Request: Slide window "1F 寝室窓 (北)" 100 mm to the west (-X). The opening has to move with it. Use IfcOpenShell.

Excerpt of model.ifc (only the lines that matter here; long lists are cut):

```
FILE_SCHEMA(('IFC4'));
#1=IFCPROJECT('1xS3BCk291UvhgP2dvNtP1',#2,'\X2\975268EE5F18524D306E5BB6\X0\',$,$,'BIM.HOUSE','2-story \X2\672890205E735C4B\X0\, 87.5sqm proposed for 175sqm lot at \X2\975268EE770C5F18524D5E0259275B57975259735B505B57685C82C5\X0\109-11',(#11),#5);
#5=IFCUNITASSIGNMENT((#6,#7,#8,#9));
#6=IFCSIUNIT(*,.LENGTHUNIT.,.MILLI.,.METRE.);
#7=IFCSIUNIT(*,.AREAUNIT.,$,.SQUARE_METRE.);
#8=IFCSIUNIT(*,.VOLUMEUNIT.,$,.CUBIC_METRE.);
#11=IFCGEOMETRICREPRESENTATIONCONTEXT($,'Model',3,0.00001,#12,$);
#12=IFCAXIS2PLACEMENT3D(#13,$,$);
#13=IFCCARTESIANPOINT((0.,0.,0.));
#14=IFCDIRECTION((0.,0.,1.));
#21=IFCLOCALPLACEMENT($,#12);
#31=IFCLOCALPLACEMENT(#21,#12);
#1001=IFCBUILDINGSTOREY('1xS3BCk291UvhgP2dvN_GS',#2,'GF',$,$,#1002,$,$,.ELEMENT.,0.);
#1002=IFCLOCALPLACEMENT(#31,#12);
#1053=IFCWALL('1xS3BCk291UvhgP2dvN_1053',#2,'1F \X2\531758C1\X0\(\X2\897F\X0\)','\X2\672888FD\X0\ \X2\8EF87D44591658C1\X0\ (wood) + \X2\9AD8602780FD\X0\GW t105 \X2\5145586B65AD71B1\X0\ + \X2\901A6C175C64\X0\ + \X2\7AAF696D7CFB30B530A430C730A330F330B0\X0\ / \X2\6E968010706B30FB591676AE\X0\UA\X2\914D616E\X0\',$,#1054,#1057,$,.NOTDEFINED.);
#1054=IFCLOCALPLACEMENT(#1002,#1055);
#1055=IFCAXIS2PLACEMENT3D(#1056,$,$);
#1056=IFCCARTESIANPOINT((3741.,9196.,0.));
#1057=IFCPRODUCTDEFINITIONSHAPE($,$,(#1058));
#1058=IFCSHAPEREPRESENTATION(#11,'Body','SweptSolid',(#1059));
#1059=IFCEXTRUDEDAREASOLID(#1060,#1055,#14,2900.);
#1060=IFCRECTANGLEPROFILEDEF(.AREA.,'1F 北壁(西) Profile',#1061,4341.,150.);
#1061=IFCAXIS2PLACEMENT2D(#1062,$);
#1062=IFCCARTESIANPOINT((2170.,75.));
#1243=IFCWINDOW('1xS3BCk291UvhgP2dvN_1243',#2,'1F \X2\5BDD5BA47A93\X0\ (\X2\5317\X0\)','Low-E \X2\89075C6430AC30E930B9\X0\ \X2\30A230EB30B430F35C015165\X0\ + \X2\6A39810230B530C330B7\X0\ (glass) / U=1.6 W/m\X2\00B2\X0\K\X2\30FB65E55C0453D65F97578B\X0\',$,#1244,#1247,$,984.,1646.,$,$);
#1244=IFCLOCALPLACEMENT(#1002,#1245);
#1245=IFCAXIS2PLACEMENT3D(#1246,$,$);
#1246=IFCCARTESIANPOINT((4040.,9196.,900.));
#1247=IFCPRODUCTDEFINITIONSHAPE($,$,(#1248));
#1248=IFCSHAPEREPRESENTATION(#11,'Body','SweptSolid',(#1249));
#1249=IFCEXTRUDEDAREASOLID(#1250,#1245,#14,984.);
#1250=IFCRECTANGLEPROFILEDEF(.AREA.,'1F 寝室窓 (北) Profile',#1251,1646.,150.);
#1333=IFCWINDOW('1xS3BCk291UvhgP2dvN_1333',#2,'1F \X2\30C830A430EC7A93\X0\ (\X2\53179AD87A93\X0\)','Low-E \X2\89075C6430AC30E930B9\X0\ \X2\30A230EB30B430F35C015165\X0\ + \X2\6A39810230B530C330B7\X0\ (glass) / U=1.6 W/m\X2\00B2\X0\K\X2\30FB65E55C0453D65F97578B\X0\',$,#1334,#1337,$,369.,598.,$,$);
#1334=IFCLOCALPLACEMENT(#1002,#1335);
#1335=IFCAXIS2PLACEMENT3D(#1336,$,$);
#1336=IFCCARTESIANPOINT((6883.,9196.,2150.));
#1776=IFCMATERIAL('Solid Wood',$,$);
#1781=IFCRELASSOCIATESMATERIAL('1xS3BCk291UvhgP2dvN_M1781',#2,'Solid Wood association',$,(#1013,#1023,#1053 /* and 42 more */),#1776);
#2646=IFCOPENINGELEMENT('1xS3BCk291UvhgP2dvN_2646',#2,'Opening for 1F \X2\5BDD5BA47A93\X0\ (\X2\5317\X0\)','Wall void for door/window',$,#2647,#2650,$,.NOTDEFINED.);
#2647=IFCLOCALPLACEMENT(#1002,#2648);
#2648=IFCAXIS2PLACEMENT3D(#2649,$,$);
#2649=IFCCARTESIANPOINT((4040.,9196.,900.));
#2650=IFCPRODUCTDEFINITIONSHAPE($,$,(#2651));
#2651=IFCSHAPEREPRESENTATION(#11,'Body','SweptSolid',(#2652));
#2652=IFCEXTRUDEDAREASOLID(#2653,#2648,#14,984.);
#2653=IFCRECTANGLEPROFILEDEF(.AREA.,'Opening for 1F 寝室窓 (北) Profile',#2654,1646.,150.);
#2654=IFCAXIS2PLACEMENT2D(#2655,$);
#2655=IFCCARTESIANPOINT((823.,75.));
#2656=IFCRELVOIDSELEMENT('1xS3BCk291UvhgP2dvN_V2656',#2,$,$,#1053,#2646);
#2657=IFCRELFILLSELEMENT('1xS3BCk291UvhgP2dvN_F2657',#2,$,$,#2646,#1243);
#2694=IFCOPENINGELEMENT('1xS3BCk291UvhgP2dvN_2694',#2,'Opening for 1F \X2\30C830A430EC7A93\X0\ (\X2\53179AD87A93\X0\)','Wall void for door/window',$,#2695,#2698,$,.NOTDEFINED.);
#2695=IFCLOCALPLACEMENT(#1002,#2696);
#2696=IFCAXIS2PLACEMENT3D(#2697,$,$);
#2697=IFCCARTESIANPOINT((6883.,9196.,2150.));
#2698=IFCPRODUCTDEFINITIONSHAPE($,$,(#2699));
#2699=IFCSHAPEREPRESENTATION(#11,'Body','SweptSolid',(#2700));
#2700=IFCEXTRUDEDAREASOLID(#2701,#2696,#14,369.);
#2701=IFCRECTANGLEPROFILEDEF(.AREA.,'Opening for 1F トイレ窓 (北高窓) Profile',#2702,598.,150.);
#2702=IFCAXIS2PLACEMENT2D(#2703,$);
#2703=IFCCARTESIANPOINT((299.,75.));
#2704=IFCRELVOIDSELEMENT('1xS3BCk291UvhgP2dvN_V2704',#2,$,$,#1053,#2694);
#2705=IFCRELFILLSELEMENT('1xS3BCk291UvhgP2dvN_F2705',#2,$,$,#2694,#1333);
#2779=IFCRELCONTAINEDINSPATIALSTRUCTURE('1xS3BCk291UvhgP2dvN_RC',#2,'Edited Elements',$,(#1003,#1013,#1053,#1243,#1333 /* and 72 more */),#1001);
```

```python
import ifcopenshell
import ifcopenshell.api.geometry
import ifcopenshell.util.placement
import ifcopenshell.util.unit

model = ifcopenshell.open("model.ifc")
unit_scale = ifcopenshell.util.unit.calculate_unit_scale(model)

window = model.by_id(1243)
opening = window.FillsVoids[0].RelatingOpeningElement
wall = opening.VoidsElements[0].RelatingBuildingElement

wall_matrix = ifcopenshell.util.placement.get_local_placement(wall.ObjectPlacement)
shift = wall_matrix[:3, 0] * -0.1 / unit_scale
before = ifcopenshell.util.placement.get_local_placement(window.ObjectPlacement)[:3, 3].copy()

# The window is not placed relative to its opening, so move both.
for product in (opening, window):
    matrix = ifcopenshell.util.placement.get_local_placement(product.ObjectPlacement)
    matrix[:3, 3] += shift
    ifcopenshell.api.geometry.edit_object_placement(model, product=product, matrix=matrix, is_si=False)

after = ifcopenshell.util.placement.get_local_placement(window.ObjectPlacement)[:3, 3]
print("window moved by", (after - before).round(3) + 0.0)

model.write("model_rev.ifc")
```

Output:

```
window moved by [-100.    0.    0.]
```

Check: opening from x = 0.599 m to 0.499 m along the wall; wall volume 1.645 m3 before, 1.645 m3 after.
